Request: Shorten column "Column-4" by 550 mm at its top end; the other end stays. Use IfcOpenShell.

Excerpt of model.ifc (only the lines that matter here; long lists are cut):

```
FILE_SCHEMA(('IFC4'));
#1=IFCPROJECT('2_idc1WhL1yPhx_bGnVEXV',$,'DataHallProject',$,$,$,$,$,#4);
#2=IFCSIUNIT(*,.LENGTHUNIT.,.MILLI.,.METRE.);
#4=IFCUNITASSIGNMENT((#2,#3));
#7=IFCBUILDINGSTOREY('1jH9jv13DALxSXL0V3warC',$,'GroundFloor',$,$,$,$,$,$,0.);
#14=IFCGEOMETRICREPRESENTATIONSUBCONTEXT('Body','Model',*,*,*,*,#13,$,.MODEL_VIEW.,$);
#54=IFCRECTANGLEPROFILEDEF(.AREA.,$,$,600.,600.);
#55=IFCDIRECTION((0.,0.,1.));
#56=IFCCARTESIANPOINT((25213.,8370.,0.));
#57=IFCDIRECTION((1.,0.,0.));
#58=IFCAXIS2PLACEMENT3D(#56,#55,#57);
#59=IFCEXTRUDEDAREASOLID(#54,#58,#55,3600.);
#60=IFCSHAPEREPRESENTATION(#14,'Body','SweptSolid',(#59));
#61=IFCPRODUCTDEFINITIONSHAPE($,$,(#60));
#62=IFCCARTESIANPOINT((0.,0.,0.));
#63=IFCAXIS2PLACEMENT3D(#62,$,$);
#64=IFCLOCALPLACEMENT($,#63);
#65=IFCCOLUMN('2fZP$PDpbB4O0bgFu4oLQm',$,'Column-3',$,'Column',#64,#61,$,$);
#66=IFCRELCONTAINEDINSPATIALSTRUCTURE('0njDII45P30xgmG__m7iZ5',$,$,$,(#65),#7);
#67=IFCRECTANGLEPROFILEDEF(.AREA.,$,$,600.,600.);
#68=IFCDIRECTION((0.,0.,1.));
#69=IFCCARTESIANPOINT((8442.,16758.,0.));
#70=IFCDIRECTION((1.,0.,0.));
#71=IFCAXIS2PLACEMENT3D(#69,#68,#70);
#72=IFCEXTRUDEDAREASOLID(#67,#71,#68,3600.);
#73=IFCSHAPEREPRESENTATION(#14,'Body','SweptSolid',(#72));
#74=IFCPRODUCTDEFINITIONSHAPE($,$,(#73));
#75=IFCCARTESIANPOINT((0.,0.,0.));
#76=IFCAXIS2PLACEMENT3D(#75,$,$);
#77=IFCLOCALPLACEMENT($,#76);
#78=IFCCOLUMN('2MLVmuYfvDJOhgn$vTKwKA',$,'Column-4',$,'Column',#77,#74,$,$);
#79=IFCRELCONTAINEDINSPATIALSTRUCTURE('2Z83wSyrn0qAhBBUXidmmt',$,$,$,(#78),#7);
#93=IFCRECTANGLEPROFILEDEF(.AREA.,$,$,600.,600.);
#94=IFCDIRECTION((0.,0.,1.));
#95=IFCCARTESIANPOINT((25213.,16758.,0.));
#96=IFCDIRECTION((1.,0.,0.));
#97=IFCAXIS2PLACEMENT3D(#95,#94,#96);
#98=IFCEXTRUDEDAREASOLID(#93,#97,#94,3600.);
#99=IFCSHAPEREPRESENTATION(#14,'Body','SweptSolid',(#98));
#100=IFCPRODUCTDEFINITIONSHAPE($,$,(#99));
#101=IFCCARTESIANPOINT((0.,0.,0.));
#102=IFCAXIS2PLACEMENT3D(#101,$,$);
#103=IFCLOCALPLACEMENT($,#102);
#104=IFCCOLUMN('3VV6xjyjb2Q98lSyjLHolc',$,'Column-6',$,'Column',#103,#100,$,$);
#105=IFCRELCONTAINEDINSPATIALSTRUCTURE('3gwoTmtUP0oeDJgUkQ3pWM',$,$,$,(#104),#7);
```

```python
import ifcopenshell
import ifcopenshell.util.representation

model = ifcopenshell.open("model.ifc")

member = model.by_id(78)
change = -550.0

# The extrusion runs towards the end named, so only its depth changes.
body = ifcopenshell.util.representation.get_representation(member, "Model", "Body")
solid = body.Items[0]
old_length = solid.Depth
solid.Depth += change

print(f"length {old_length:g} -> {solid.Depth:g}")

model.write("model_edited.ifc")
```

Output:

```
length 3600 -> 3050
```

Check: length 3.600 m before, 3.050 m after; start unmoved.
